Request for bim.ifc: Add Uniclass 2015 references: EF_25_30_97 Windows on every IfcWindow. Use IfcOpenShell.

First a look at what the model holds.

```python
import ifcopenshell

model = ifcopenshell.open("bim.ifc")
print(model.schema)
print("classifications:", [c.Name for c in model.by_type("IfcClassification")])
for ifc_class in ("IfcDoor", "IfcRoof", "IfcStair", "IfcWall", "IfcWindow"):
    print(ifc_class, len(model.by_type(ifc_class)))
```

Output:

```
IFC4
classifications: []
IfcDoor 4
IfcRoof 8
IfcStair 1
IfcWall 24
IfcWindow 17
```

```python
import ifcopenshell
import ifcopenshell.api.classification

model = ifcopenshell.open("bim.ifc")

system = ifcopenshell.api.classification.add_classification(model, classification="Uniclass 2015")

codes = {
    "IfcWindow": ("EF_25_30_97", "Windows"),
}
for ifc_class, (code, name) in codes.items():
    products = model.by_type(ifc_class)
    ifcopenshell.api.classification.add_reference(
        model, products=products, classification=system, identification=code, name=name
    )
    print(code, len(products))

model.write("bim_rev.ifc")
```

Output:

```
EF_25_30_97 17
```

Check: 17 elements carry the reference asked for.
